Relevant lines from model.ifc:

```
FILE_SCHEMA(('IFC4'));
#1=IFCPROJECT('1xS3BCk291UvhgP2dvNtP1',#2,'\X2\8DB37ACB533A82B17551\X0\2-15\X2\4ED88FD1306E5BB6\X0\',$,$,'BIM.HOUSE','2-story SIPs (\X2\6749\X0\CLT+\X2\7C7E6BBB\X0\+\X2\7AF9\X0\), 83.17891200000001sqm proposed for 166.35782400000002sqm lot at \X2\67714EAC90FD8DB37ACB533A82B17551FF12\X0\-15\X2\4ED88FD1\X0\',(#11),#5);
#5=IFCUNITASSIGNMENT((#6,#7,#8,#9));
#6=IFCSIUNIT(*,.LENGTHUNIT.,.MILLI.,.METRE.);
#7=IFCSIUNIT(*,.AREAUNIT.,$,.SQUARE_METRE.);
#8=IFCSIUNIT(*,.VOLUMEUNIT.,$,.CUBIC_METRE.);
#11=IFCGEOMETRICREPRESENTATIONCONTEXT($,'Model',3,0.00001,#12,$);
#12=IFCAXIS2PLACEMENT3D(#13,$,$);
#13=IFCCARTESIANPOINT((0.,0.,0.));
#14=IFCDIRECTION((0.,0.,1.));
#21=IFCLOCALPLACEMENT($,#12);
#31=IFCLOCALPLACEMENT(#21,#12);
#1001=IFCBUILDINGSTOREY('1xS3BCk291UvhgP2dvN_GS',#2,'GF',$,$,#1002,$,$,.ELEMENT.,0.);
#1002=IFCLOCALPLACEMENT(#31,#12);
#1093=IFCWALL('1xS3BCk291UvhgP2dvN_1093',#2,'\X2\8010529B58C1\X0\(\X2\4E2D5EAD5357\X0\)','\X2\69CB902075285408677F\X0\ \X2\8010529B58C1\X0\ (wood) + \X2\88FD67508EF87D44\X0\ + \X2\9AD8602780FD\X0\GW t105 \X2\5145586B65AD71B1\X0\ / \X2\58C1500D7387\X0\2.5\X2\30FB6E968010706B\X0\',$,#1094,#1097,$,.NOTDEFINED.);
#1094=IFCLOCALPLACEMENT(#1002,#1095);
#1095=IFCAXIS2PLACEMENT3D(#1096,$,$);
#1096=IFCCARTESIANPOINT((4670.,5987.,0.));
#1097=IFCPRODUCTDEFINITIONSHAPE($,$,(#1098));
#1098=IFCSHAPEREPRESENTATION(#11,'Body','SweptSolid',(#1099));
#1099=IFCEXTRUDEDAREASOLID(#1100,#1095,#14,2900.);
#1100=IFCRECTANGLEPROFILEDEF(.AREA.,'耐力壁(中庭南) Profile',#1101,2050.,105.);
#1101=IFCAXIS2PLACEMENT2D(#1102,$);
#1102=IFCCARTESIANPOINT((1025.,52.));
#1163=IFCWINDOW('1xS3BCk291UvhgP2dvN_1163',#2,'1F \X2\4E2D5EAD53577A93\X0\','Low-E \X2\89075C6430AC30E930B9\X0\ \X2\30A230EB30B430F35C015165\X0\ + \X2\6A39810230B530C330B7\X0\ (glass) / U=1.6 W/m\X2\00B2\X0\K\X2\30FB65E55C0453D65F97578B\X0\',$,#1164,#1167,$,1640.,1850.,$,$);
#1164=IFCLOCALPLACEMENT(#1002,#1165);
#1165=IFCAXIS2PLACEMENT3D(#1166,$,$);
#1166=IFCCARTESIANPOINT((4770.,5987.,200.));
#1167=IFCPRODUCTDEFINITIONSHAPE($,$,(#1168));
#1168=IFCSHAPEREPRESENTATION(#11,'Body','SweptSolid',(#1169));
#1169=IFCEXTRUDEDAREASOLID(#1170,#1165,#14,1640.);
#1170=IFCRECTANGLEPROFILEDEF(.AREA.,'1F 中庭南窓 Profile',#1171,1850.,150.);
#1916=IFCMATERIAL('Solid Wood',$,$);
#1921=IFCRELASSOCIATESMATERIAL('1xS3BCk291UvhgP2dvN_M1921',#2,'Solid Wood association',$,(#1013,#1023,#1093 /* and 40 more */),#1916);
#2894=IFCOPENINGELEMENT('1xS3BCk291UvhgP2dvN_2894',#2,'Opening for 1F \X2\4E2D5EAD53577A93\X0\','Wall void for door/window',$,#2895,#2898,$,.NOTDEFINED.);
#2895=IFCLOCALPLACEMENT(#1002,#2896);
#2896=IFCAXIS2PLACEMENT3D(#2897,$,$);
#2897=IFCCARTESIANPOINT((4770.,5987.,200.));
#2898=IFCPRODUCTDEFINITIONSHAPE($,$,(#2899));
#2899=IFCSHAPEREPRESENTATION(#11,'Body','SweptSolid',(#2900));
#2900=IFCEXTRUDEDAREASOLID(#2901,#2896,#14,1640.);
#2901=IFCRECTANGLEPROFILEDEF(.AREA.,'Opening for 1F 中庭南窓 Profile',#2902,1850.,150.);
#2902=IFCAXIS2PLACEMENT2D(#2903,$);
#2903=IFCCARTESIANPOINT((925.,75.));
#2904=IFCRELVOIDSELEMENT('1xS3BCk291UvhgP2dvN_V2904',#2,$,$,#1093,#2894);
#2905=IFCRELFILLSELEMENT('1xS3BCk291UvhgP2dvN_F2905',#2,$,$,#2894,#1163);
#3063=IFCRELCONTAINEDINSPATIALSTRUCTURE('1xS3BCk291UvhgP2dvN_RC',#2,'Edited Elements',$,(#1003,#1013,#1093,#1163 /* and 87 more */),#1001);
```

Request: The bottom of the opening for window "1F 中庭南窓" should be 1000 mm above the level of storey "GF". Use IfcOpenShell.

```python
import numpy as np
import ifcopenshell
import ifcopenshell.api.geometry
import ifcopenshell.geom
import ifcopenshell.util.element
import ifcopenshell.util.placement
import ifcopenshell.util.shape
import ifcopenshell.util.unit

model = ifcopenshell.open("model.ifc")
unit_scale = ifcopenshell.util.unit.calculate_unit_scale(model)

window = model.by_guid("1xS3BCk291UvhgP2dvN_1163")
opening = window.FillsVoids[0].RelatingOpeningElement
storey = ifcopenshell.util.element.get_container(window, ifc_class="IfcBuildingStorey")
level = ifcopenshell.util.placement.get_local_placement(storey.ObjectPlacement)[2, 3]

# The opening's origin need not be at the sill, so measure its lowest point.
shape = ifcopenshell.geom.create_shape(ifcopenshell.geom.settings(), opening)
bottom = ifcopenshell.util.shape.get_shape_bottom_elevation(shape, shape.geometry) / unit_scale
dz = level + 1 / unit_scale - bottom

shift = np.array([0.0, 0.0, dz])
# The window is not placed relative to its opening, so move both.
for product in (opening, window):
    matrix = ifcopenshell.util.placement.get_local_placement(product.ObjectPlacement)
    matrix[:3, 3] += shift
    ifcopenshell.api.geometry.edit_object_placement(model, product=product, matrix=matrix, is_si=False)

print(f"moved by {dz * unit_scale:+.3f} m")

model.write("model_edited.ifc")
```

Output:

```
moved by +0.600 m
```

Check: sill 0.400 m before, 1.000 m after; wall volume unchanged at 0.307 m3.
